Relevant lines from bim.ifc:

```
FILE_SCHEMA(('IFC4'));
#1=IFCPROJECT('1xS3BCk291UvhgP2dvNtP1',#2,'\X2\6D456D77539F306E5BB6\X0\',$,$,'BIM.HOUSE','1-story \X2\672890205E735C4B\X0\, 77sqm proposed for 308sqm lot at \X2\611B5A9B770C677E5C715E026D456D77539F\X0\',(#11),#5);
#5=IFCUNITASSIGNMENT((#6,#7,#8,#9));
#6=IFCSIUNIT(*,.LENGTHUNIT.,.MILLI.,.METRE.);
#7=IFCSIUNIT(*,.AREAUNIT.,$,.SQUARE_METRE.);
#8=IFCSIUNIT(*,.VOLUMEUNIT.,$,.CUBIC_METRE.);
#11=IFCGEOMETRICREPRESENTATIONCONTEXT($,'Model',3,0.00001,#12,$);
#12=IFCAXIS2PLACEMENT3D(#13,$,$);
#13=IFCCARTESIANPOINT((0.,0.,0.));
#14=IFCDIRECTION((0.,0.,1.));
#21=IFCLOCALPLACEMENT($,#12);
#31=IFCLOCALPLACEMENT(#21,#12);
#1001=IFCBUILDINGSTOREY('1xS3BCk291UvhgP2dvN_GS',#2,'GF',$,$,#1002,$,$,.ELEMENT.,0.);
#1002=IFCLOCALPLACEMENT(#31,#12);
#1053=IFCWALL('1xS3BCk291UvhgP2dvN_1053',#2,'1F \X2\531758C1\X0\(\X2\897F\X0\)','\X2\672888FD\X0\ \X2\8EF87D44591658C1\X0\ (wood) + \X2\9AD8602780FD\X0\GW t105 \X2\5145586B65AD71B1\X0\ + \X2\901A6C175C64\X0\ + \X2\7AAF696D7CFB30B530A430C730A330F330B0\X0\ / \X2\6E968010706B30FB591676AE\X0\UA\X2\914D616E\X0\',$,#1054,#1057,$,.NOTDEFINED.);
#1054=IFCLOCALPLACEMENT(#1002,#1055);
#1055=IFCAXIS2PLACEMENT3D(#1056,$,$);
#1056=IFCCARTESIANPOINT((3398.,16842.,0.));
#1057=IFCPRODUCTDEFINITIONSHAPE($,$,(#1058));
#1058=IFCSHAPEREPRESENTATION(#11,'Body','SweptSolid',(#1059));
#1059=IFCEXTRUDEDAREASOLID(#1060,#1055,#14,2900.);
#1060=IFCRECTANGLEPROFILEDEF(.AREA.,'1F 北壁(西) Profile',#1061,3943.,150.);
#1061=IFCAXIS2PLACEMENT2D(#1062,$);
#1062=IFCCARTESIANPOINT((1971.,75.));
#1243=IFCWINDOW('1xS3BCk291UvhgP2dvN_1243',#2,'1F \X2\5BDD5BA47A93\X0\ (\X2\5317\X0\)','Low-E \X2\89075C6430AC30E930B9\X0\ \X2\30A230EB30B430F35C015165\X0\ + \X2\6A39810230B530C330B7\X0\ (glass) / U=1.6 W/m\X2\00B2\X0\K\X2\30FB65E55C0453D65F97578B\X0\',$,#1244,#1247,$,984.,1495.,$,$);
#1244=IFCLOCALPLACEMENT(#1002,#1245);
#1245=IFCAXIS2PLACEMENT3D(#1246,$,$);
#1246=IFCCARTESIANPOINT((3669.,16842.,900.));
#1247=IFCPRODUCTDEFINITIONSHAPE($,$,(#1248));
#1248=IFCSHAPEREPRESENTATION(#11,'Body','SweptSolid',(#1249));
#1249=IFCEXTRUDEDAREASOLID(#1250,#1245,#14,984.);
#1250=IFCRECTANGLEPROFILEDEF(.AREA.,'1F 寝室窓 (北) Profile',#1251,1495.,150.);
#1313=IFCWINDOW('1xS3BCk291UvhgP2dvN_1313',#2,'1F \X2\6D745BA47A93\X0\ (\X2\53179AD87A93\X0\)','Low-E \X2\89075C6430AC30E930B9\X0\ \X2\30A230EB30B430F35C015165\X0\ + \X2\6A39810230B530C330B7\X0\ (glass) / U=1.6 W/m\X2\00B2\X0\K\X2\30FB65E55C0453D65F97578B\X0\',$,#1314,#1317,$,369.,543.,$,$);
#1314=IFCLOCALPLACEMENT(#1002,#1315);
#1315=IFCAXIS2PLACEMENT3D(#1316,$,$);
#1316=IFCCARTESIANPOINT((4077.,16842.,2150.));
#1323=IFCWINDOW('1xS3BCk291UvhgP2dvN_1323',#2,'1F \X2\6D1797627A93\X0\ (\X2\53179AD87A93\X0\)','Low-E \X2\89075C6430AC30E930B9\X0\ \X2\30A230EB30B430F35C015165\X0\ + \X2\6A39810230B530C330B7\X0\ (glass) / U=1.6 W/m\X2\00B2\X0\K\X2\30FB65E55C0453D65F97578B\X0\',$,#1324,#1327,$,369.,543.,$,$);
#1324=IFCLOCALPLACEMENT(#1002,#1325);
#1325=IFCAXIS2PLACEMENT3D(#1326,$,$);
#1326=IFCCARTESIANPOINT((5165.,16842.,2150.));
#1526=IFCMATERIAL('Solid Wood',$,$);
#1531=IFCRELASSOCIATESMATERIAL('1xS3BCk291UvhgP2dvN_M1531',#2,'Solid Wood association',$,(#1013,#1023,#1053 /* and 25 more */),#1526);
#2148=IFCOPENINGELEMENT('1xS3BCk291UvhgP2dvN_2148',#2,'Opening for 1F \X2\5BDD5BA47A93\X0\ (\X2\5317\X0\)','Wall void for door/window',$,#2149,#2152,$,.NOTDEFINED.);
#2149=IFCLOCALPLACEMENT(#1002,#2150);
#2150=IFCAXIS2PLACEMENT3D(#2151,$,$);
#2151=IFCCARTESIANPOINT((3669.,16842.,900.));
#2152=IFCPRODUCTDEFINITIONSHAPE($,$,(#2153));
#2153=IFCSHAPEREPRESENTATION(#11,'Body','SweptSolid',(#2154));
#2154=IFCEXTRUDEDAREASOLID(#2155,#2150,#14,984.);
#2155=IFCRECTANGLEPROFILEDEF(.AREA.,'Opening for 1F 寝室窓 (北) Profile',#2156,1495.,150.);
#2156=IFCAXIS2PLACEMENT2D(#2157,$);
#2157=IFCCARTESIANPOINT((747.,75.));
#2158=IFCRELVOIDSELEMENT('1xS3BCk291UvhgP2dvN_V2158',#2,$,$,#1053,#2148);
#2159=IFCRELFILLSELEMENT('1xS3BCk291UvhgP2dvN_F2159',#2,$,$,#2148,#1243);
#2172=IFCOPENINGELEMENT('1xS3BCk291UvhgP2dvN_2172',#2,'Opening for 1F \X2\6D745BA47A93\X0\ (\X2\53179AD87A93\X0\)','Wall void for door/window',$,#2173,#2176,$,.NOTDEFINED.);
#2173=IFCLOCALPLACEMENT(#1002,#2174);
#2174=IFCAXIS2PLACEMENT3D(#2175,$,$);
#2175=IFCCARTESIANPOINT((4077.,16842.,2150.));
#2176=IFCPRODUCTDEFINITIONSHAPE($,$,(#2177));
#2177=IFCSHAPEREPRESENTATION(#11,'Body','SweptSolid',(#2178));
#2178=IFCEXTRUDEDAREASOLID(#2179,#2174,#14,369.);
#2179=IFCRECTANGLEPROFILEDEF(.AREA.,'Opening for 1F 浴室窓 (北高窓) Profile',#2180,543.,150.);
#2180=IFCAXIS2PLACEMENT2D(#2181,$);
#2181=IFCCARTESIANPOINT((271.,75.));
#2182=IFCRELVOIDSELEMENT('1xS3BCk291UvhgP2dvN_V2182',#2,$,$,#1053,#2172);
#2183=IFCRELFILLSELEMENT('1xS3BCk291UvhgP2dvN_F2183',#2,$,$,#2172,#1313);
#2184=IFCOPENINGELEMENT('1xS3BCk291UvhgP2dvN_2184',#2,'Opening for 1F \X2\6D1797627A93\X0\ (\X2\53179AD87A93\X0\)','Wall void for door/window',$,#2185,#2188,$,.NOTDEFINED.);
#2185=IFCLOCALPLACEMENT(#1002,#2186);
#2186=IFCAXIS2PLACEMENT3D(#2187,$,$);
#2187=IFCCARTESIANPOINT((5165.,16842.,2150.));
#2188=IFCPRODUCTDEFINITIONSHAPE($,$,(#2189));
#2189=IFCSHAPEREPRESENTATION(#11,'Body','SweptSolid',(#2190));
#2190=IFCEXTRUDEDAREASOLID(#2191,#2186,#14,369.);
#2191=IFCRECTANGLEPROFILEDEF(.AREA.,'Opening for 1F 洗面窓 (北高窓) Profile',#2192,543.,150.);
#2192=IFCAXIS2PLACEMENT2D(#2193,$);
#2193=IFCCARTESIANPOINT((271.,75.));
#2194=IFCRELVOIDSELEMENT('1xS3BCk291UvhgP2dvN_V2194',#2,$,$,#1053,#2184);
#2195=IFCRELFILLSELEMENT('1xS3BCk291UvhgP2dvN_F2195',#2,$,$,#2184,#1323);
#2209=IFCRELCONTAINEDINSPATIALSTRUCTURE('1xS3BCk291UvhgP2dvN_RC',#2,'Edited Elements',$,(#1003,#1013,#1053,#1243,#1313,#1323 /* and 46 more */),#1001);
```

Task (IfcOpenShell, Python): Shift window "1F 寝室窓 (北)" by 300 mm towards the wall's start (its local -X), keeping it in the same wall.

```python
import ifcopenshell
import ifcopenshell.api.geometry
import ifcopenshell.util.placement
import ifcopenshell.util.unit

model = ifcopenshell.open("bim.ifc")
unit_scale = ifcopenshell.util.unit.calculate_unit_scale(model)

window = model.by_guid("1xS3BCk291UvhgP2dvN_1243")
opening = window.FillsVoids[0].RelatingOpeningElement
wall = opening.VoidsElements[0].RelatingBuildingElement

wall_matrix = ifcopenshell.util.placement.get_local_placement(wall.ObjectPlacement)
shift = wall_matrix[:3, 0] * -0.3 / unit_scale
before = ifcopenshell.util.placement.get_local_placement(window.ObjectPlacement)[:3, 3].copy()

# The window is not placed relative to its opening, so move both.
for product in (opening, window):
    matrix = ifcopenshell.util.placement.get_local_placement(product.ObjectPlacement)
    matrix[:3, 3] += shift
    ifcopenshell.api.geometry.edit_object_placement(model, product=product, matrix=matrix, is_si=False)

after = ifcopenshell.util.placement.get_local_placement(window.ObjectPlacement)[:3, 3]
print("window moved by", (after - before).round(3) + 0.0)

model.write("bim_v2.ifc")
```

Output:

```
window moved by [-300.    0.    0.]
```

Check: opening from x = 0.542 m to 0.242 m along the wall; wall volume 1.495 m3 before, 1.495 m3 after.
